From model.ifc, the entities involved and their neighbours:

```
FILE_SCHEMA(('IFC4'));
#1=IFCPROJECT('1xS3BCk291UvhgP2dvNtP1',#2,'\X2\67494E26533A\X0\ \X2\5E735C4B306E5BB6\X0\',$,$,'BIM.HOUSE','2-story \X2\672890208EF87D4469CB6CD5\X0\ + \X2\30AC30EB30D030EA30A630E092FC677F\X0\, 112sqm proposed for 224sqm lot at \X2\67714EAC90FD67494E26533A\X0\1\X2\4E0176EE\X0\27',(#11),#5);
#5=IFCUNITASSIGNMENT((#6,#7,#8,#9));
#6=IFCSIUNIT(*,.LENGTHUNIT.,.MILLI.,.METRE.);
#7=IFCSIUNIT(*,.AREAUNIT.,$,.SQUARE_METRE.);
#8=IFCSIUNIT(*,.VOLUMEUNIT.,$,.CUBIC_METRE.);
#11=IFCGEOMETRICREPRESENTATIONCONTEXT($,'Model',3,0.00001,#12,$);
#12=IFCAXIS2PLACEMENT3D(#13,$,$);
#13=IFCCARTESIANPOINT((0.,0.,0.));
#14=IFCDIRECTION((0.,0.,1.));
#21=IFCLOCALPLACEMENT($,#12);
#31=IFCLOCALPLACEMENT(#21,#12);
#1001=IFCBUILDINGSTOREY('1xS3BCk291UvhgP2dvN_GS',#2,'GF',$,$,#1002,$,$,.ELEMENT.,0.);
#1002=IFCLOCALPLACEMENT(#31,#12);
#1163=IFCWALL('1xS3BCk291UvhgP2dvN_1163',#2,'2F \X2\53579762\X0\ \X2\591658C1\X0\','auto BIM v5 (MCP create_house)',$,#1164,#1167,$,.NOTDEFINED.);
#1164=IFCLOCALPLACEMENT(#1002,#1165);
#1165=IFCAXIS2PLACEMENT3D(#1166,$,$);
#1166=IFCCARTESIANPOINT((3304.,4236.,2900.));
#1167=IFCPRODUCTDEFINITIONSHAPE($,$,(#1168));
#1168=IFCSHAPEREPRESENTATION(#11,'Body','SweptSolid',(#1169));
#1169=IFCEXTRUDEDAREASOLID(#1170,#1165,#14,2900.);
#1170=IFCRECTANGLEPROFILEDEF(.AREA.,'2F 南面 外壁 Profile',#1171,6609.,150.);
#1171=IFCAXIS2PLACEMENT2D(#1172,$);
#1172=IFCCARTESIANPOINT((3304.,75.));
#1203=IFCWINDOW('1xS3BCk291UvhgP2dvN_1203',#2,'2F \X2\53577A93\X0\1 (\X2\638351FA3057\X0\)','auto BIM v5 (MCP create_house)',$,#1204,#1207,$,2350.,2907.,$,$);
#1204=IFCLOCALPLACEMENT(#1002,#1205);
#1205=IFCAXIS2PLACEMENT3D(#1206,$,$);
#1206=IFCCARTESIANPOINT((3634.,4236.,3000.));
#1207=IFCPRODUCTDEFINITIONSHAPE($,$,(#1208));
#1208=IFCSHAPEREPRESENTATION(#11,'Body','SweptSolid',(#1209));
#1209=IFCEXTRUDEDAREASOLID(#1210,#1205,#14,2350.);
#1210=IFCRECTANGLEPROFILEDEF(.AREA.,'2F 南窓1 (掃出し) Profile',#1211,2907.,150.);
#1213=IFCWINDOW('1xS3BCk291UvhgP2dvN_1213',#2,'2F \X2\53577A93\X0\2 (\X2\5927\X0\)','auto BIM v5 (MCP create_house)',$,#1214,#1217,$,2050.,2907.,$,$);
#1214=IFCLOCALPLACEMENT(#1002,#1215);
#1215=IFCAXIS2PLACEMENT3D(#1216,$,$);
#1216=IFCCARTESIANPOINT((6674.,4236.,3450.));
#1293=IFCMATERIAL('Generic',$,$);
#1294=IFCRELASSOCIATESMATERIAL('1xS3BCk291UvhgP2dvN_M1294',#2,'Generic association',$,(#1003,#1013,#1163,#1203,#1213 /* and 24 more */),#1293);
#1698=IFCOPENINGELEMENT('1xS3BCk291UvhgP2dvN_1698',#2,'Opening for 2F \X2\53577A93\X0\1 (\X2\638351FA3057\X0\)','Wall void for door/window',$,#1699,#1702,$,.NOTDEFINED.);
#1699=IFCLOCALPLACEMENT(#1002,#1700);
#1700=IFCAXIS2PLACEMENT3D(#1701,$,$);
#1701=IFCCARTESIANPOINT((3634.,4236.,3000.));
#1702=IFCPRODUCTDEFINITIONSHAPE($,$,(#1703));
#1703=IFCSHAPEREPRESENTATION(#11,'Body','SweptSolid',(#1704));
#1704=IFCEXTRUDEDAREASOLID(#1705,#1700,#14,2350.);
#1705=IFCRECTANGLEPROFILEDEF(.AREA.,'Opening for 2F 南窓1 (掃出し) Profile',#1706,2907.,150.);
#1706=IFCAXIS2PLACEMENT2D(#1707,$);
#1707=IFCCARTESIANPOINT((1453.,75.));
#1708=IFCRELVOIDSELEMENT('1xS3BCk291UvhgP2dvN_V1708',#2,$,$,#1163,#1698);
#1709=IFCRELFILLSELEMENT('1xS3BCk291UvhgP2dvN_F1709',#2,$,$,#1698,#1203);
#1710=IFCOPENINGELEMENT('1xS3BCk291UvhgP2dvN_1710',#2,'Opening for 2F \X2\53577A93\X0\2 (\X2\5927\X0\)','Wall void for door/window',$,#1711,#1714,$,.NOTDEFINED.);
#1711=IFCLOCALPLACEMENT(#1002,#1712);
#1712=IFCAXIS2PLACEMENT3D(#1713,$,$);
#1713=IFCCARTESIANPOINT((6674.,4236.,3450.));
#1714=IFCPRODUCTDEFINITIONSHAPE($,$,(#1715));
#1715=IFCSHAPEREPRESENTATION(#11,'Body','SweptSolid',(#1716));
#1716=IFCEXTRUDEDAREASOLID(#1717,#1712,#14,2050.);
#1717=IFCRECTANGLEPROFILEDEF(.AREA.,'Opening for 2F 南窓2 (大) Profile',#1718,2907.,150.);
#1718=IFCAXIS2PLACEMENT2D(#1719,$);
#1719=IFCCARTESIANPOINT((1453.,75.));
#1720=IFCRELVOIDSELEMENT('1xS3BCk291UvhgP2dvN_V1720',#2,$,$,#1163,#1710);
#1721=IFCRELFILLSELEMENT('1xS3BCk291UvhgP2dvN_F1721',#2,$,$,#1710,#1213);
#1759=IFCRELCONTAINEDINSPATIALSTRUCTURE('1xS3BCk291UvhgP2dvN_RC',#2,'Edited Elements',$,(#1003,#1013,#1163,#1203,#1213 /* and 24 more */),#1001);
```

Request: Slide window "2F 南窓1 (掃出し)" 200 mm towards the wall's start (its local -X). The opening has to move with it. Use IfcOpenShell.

```python
import ifcopenshell
import ifcopenshell.api.geometry
import ifcopenshell.util.placement

model = ifcopenshell.open("model.ifc")

window = model.by_id(1203)
opening = window.FillsVoids[0].RelatingOpeningElement
wall = opening.VoidsElements[0].RelatingBuildingElement

wall_matrix = ifcopenshell.util.placement.get_local_placement(wall.ObjectPlacement)
shift = wall_matrix[:3, 0] * -200.0
before = ifcopenshell.util.placement.get_local_placement(window.ObjectPlacement)[:3, 3].copy()

# The window is not placed relative to its opening, so move both.
for product in (opening, window):
    matrix = ifcopenshell.util.placement.get_local_placement(product.ObjectPlacement)
    matrix[:3, 3] += shift
    ifcopenshell.api.geometry.edit_object_placement(model, product=product, matrix=matrix, is_si=False)

after = ifcopenshell.util.placement.get_local_placement(window.ObjectPlacement)[:3, 3]
print("window moved by", (after - before).round(3) + 0.0)

model.write("model-out.ifc")
```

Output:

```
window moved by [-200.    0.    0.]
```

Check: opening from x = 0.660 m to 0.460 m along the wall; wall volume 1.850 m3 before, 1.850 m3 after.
